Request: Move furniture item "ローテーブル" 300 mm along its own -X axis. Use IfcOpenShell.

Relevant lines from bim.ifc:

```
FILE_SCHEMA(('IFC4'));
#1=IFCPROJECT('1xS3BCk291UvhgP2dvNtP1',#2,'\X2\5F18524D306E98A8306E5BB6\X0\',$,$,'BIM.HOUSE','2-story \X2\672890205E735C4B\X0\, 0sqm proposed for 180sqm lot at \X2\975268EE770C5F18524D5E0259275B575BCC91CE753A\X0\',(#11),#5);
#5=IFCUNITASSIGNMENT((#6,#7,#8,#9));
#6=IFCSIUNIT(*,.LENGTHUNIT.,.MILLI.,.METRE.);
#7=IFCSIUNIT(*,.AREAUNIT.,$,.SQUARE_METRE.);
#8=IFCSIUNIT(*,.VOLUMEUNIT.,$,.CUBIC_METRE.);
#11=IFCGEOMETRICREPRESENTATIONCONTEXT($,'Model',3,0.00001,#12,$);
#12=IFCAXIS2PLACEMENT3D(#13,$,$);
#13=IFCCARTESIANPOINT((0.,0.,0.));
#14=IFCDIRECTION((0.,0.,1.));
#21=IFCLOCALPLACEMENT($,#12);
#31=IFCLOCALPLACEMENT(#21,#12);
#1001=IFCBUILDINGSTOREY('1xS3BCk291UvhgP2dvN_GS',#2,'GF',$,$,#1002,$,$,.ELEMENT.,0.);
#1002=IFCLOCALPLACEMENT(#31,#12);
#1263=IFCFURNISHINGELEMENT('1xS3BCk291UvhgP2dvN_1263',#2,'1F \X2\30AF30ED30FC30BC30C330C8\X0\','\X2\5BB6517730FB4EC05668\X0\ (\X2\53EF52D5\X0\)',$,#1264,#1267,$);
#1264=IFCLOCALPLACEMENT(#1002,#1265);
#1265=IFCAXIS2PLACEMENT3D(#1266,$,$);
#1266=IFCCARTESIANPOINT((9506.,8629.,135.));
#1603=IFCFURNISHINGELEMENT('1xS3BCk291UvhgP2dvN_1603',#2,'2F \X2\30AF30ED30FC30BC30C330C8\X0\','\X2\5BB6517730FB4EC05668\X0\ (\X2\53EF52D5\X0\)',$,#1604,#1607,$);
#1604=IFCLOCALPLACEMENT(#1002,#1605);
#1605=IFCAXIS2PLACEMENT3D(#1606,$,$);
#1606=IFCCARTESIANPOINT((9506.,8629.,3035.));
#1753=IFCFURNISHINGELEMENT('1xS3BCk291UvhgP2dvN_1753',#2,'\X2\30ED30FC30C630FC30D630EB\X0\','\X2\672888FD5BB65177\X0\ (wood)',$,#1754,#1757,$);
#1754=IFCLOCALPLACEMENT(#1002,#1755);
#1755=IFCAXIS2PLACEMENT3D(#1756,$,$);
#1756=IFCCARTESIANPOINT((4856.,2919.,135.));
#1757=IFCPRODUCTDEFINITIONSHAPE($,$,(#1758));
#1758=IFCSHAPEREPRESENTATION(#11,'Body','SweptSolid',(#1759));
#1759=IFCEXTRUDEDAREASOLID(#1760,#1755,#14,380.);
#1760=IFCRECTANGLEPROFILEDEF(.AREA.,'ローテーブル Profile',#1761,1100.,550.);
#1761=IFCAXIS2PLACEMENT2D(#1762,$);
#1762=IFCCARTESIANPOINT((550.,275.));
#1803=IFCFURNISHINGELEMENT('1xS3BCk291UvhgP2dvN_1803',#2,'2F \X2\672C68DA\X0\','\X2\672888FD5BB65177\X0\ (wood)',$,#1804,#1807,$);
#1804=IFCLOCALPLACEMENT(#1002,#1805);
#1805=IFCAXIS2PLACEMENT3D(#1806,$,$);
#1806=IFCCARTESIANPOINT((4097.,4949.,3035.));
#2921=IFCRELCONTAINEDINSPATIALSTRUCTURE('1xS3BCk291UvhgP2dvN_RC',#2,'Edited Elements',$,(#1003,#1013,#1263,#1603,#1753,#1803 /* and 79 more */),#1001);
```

```python
import ifcopenshell
import ifcopenshell.api.geometry
import ifcopenshell.util.placement

model = ifcopenshell.open("bim.ifc")

item = model.by_guid("1xS3BCk291UvhgP2dvN_1753")
matrix = ifcopenshell.util.placement.get_local_placement(item.ObjectPlacement)
matrix[:3, 3] -= matrix[:3, 0] * 300.0
ifcopenshell.api.geometry.edit_object_placement(model, product=item, matrix=matrix, is_si=False)

print(ifcopenshell.util.placement.get_local_placement(item.ObjectPlacement).round(3) + 0.0)

model.write("bim-out.ifc")
```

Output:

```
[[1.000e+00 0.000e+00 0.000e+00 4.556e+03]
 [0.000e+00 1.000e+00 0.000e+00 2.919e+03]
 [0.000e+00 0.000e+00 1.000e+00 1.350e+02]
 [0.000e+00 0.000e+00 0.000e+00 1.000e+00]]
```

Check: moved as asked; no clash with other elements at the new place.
